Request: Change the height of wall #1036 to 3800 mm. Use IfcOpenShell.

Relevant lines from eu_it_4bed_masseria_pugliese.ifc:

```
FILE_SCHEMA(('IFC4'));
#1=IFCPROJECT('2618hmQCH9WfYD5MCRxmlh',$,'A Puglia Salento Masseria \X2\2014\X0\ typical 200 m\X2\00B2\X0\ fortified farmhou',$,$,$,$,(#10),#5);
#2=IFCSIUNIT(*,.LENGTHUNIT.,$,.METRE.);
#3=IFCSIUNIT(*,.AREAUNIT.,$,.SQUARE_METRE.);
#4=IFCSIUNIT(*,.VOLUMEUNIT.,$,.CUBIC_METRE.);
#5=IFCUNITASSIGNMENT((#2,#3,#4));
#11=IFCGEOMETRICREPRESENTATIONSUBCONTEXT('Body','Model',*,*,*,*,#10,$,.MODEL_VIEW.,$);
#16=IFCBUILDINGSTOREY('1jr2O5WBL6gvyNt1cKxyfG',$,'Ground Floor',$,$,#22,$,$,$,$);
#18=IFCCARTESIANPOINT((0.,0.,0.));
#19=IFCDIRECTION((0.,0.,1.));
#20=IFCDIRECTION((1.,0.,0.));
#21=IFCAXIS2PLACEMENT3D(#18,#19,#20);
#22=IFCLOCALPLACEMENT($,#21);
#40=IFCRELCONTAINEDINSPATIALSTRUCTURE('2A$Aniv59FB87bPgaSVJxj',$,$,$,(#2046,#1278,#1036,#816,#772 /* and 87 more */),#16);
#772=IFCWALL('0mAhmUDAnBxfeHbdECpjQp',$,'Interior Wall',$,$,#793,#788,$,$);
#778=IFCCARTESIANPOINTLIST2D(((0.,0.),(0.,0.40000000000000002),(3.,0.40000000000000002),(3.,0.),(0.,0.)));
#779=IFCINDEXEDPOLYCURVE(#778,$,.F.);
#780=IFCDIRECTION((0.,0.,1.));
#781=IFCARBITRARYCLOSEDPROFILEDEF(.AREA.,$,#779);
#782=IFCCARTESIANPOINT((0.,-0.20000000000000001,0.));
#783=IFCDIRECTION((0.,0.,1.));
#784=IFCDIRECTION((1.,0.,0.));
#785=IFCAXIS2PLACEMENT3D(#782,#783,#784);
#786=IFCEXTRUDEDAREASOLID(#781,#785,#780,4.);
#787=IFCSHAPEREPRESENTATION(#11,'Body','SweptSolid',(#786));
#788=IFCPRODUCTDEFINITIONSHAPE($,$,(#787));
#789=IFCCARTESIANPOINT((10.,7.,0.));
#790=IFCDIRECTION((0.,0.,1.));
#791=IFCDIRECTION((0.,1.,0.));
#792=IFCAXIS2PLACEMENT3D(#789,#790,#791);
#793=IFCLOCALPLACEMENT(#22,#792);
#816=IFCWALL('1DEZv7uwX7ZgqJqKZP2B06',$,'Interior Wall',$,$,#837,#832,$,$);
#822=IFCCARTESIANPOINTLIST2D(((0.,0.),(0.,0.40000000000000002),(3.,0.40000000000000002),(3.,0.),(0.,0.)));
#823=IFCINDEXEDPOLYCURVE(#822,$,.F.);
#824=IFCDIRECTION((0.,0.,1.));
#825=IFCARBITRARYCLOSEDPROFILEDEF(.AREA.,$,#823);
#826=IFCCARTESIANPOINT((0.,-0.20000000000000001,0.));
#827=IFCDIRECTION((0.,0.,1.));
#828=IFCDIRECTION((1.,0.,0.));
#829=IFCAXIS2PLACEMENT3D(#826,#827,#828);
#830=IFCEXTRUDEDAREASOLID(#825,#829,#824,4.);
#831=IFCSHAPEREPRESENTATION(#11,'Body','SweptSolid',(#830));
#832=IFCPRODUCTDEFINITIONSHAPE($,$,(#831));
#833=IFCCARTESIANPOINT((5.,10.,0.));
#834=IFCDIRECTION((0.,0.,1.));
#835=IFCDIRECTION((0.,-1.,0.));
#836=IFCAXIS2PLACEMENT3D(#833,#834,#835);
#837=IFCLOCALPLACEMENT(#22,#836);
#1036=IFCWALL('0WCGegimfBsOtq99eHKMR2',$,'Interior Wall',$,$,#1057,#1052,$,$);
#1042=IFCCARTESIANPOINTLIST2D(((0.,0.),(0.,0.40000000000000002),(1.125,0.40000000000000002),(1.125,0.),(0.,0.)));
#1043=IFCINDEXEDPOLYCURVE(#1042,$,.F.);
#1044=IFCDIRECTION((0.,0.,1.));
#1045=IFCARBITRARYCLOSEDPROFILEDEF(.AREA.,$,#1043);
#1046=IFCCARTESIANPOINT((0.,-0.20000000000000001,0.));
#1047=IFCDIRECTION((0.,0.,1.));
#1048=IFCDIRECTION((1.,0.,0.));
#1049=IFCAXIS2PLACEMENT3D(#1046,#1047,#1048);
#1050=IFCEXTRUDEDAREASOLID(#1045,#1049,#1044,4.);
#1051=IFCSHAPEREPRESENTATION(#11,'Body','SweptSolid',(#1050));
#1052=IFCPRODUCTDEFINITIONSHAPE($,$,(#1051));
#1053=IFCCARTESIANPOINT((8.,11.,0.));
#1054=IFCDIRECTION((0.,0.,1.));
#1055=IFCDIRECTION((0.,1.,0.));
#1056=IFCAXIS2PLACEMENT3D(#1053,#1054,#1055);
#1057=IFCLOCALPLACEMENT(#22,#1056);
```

```python
import ifcopenshell
import ifcopenshell.geom
import ifcopenshell.util.representation
import ifcopenshell.util.shape

model = ifcopenshell.open("eu_it_4bed_masseria_pugliese.ifc")
settings = ifcopenshell.geom.settings()


def volume(element):
    """Net volume in cubic metres, openings subtracted."""
    shape = ifcopenshell.geom.create_shape(settings, element)
    return ifcopenshell.util.shape.get_volume(shape.geometry)


wall = model.by_guid("0WCGegimfBsOtq99eHKMR2")
before = volume(wall)

body = ifcopenshell.util.representation.get_representation(wall, "Model", "Body")
solid = body.Items[0]
old_height = solid.Depth
solid.Depth = 3.8
after = volume(wall)

print(f"height {old_height:g} -> {solid.Depth:g}, volume {before:.3f} -> {after:.3f} m3")

model.write("eu_it_4bed_masseria_pugliese_edited.ifc")
```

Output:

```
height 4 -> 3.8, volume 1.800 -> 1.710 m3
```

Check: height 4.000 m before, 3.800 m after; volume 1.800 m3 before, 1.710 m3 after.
